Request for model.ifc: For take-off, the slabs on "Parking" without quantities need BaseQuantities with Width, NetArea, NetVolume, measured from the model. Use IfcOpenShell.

First a look at what the model holds.

```python
import ifcopenshell
import ifcopenshell.util.element
import ifcopenshell.util.unit

model = ifcopenshell.open("model.ifc")
print(model.schema)
for unit_type in ("LENGTHUNIT", "AREAUNIT", "VOLUMEUNIT"):
    print(unit_type, ifcopenshell.util.unit.calculate_unit_scale(model, unit_type))
storey = next(s for s in model.by_type("IfcBuildingStorey") if s.Name == "Parking")
slabs = [e for e in ifcopenshell.util.element.get_decomposition(storey) if e.is_a("IfcSlab")]
for e in sorted(slabs, key=lambda e: e.id()):
    print(e.id(), e.is_a(), e.Name, list(ifcopenshell.util.element.get_psets(e, qtos_only=True)), sep=" | ")
```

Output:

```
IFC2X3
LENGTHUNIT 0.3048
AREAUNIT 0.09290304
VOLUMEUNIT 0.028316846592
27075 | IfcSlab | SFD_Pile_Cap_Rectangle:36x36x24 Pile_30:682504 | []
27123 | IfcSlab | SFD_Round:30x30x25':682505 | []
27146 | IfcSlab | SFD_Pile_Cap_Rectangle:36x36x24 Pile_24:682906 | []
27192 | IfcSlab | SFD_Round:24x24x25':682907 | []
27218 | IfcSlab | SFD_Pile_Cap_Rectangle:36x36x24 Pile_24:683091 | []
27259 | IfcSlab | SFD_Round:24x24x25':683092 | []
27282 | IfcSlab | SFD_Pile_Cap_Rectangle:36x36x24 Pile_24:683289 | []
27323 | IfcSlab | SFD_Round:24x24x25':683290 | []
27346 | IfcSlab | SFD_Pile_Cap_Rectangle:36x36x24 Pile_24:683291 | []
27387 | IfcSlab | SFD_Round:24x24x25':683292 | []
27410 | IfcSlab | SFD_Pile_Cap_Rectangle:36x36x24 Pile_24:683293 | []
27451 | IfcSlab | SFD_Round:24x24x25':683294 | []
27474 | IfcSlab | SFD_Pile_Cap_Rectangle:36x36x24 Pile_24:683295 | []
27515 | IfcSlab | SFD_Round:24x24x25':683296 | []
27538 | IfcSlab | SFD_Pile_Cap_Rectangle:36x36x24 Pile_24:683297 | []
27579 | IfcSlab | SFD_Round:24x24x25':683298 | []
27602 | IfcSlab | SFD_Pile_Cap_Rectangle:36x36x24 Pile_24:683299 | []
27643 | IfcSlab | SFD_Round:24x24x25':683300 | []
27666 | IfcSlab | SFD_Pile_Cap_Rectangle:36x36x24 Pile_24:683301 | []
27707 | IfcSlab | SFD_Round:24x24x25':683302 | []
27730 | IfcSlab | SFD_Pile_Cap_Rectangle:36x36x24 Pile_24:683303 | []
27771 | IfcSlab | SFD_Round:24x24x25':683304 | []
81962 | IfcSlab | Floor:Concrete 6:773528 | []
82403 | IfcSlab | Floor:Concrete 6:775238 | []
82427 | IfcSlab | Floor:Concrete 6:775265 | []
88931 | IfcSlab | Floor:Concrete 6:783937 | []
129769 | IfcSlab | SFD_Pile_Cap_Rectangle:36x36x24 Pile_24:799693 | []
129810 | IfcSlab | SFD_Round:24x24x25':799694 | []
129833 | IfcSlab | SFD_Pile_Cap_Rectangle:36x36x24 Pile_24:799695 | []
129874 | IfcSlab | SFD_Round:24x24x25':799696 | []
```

```python
import ifcopenshell
import ifcopenshell.api.pset
import ifcopenshell.geom
import ifcopenshell.util.element
import ifcopenshell.util.shape
import ifcopenshell.util.unit

model = ifcopenshell.open("model.ifc")
unit_scale = ifcopenshell.util.unit.calculate_unit_scale(model)
area_scale = ifcopenshell.util.unit.calculate_unit_scale(model, "AREAUNIT")
volume_scale = ifcopenshell.util.unit.calculate_unit_scale(model, "VOLUMEUNIT")
settings = ifcopenshell.geom.settings()

storey = next(s for s in model.by_type("IfcBuildingStorey") if s.Name == "Parking")
slabs = [e for e in ifcopenshell.util.element.get_decomposition(storey) if e.is_a("IfcSlab")]

for e in sorted(slabs, key=lambda e: e.id()):
    if ifcopenshell.util.element.get_psets(e, qtos_only=True, should_inherit=False):
        continue
    # Geometry comes back in metres, in the element's own axes.
    shape = ifcopenshell.geom.create_shape(settings, e)
    values = {
        "Width": ifcopenshell.util.shape.get_z(shape.geometry) / unit_scale,
        "NetArea": ifcopenshell.util.shape.get_footprint_area(shape.geometry) / area_scale,
        "NetVolume": ifcopenshell.util.shape.get_volume(shape.geometry) / volume_scale,
    }
    qto = ifcopenshell.api.pset.add_qto(model, product=e, name="BaseQuantities")
    ifcopenshell.api.pset.edit_qto(model, qto=qto, properties=values)
    print(e.id(), {k: round(v, 3) for k, v in values.items()})

model.write("model_updated.ifc")
```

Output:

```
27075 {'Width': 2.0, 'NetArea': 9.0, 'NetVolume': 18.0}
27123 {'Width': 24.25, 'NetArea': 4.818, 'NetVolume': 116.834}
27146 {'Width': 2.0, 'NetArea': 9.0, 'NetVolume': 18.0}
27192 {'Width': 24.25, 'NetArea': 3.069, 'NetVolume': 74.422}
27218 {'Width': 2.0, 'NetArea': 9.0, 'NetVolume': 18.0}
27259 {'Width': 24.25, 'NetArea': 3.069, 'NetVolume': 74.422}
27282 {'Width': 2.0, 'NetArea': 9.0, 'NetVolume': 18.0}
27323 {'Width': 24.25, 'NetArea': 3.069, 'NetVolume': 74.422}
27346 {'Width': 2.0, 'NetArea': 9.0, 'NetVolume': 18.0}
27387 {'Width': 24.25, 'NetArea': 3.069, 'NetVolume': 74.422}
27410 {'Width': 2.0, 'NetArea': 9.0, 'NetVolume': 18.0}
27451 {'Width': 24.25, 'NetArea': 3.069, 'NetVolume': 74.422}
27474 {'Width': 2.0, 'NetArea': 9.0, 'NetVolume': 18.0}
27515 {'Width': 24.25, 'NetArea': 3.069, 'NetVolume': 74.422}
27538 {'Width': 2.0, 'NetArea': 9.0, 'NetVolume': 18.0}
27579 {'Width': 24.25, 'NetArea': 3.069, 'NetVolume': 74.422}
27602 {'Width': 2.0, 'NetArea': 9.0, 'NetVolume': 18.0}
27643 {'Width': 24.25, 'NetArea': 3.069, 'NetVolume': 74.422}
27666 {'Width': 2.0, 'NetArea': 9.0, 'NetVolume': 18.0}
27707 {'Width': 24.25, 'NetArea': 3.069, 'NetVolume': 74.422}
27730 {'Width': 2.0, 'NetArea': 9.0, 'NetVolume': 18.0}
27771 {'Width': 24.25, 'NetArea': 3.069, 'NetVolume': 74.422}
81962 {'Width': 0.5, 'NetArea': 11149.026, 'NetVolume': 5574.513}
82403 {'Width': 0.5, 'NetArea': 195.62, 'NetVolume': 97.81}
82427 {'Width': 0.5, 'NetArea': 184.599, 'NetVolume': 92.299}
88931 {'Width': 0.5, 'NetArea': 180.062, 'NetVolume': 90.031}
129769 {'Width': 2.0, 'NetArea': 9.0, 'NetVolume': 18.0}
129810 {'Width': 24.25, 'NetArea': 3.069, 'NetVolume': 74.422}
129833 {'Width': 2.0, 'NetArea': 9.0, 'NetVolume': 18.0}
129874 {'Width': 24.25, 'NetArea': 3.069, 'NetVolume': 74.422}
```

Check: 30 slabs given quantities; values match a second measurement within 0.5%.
